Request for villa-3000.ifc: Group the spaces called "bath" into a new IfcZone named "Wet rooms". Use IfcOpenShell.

First a look at what the model holds.

```python
import ifcopenshell

model = ifcopenshell.open("villa-3000.ifc")
print(model.schema)
seen = {}
for space in model.by_type("IfcSpace"):
    seen[space.LongName] = seen.get(space.LongName, 0) + 1
for name, count in sorted(seen.items(), key=str):
    print(count, "x", name)
print("zones:", [z.Name for z in model.by_type("IfcZone")][:20])
```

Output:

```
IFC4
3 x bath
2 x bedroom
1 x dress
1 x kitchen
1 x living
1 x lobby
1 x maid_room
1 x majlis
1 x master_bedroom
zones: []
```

```python
import ifcopenshell
import ifcopenshell.api.group
import ifcopenshell.api.root

model = ifcopenshell.open("villa-3000.ifc")

names = {"bath"}
spaces = [s for s in model.by_type("IfcSpace") if s.LongName in names]

zone = ifcopenshell.api.root.create_entity(model, ifc_class="IfcZone", name="Wet rooms")
ifcopenshell.api.group.assign_group(model, products=spaces, group=zone)
print(len(spaces), "spaces in", zone.Name)

model.write("villa-3000_edited.ifc")
```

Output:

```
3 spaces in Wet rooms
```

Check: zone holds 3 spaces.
